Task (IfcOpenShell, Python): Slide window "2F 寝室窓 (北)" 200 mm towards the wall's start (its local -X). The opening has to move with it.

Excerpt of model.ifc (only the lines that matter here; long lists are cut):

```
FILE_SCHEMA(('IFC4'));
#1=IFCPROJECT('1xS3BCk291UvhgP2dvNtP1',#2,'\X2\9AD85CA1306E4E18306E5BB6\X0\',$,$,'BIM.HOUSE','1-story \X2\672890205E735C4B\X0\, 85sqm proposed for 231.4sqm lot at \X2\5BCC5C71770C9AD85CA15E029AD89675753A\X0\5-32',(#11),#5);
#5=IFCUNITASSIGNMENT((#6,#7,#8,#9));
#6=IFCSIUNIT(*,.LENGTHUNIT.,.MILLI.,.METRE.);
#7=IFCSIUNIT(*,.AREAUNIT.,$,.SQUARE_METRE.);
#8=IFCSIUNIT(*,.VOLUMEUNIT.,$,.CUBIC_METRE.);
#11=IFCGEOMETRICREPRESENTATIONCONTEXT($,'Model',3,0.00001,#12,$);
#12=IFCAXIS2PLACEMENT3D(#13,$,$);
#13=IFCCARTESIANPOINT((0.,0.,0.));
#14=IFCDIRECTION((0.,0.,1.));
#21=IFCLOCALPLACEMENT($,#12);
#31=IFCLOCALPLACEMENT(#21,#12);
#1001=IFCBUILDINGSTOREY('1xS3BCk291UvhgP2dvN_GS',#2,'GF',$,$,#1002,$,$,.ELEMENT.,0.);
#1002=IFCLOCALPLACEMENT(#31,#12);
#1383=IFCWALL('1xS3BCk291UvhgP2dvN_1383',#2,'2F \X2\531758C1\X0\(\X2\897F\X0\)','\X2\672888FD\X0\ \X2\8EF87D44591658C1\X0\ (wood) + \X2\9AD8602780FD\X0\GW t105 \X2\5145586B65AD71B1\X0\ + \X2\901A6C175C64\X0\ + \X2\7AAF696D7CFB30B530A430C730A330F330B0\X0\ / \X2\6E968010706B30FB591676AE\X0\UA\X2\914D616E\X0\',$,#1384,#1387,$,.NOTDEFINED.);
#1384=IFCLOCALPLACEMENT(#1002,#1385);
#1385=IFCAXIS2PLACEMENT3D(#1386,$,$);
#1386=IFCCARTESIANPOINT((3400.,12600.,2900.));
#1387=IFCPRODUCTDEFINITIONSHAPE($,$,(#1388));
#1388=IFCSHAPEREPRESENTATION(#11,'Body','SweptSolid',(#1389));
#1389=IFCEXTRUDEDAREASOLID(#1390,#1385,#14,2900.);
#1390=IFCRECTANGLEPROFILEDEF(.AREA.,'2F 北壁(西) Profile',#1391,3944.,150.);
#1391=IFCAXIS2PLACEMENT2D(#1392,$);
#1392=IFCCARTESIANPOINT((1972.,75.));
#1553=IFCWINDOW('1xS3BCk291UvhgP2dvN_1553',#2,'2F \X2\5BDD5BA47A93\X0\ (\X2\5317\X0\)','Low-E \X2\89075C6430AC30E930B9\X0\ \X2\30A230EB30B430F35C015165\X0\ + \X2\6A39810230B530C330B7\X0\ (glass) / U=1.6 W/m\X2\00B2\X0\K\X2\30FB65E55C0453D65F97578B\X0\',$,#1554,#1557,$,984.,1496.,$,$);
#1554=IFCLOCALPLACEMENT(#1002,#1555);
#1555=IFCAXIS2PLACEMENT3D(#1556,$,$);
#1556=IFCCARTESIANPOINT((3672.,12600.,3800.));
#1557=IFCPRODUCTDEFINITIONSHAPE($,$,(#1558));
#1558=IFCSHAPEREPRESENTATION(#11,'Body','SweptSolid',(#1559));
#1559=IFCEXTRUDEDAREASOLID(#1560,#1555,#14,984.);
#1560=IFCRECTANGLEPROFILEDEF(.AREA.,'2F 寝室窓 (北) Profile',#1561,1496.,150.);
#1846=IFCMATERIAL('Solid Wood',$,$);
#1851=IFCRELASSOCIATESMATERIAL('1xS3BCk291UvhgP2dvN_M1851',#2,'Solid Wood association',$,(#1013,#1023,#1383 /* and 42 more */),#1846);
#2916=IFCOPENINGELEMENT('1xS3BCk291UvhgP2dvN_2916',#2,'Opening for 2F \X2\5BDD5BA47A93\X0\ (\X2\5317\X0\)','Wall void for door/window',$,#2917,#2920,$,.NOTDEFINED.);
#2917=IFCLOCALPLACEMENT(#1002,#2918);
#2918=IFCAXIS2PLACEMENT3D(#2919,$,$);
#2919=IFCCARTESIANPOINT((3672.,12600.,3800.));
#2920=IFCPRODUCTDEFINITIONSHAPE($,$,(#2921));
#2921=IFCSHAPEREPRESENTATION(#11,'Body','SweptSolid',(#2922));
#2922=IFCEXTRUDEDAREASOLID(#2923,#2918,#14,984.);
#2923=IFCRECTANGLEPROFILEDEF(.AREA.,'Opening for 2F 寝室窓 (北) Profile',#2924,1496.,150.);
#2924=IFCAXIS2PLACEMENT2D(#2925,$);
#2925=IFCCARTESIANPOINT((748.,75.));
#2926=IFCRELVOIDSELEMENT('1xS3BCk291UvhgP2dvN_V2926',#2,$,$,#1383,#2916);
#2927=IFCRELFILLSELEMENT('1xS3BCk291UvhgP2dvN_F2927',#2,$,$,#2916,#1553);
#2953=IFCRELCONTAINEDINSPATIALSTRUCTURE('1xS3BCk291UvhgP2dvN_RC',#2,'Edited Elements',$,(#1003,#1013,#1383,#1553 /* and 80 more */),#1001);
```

```python
import ifcopenshell
import ifcopenshell.api.geometry
import ifcopenshell.util.placement

model = ifcopenshell.open("model.ifc")

window = model.by_guid("1xS3BCk291UvhgP2dvN_1553")
opening = window.FillsVoids[0].RelatingOpeningElement
wall = opening.VoidsElements[0].RelatingBuildingElement

wall_matrix = ifcopenshell.util.placement.get_local_placement(wall.ObjectPlacement)
shift = wall_matrix[:3, 0] * -200.0
before = ifcopenshell.util.placement.get_local_placement(window.ObjectPlacement)[:3, 3].copy()

# The window is not placed relative to its opening, so move both.
for product in (opening, window):
    matrix = ifcopenshell.util.placement.get_local_placement(product.ObjectPlacement)
    matrix[:3, 3] += shift
    ifcopenshell.api.geometry.edit_object_placement(model, product=product, matrix=matrix, is_si=False)

after = ifcopenshell.util.placement.get_local_placement(window.ObjectPlacement)[:3, 3]
print("window moved by", (after - before).round(3) + 0.0)

model.write("model-out.ifc")
```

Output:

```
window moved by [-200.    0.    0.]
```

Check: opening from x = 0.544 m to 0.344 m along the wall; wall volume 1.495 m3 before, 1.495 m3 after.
